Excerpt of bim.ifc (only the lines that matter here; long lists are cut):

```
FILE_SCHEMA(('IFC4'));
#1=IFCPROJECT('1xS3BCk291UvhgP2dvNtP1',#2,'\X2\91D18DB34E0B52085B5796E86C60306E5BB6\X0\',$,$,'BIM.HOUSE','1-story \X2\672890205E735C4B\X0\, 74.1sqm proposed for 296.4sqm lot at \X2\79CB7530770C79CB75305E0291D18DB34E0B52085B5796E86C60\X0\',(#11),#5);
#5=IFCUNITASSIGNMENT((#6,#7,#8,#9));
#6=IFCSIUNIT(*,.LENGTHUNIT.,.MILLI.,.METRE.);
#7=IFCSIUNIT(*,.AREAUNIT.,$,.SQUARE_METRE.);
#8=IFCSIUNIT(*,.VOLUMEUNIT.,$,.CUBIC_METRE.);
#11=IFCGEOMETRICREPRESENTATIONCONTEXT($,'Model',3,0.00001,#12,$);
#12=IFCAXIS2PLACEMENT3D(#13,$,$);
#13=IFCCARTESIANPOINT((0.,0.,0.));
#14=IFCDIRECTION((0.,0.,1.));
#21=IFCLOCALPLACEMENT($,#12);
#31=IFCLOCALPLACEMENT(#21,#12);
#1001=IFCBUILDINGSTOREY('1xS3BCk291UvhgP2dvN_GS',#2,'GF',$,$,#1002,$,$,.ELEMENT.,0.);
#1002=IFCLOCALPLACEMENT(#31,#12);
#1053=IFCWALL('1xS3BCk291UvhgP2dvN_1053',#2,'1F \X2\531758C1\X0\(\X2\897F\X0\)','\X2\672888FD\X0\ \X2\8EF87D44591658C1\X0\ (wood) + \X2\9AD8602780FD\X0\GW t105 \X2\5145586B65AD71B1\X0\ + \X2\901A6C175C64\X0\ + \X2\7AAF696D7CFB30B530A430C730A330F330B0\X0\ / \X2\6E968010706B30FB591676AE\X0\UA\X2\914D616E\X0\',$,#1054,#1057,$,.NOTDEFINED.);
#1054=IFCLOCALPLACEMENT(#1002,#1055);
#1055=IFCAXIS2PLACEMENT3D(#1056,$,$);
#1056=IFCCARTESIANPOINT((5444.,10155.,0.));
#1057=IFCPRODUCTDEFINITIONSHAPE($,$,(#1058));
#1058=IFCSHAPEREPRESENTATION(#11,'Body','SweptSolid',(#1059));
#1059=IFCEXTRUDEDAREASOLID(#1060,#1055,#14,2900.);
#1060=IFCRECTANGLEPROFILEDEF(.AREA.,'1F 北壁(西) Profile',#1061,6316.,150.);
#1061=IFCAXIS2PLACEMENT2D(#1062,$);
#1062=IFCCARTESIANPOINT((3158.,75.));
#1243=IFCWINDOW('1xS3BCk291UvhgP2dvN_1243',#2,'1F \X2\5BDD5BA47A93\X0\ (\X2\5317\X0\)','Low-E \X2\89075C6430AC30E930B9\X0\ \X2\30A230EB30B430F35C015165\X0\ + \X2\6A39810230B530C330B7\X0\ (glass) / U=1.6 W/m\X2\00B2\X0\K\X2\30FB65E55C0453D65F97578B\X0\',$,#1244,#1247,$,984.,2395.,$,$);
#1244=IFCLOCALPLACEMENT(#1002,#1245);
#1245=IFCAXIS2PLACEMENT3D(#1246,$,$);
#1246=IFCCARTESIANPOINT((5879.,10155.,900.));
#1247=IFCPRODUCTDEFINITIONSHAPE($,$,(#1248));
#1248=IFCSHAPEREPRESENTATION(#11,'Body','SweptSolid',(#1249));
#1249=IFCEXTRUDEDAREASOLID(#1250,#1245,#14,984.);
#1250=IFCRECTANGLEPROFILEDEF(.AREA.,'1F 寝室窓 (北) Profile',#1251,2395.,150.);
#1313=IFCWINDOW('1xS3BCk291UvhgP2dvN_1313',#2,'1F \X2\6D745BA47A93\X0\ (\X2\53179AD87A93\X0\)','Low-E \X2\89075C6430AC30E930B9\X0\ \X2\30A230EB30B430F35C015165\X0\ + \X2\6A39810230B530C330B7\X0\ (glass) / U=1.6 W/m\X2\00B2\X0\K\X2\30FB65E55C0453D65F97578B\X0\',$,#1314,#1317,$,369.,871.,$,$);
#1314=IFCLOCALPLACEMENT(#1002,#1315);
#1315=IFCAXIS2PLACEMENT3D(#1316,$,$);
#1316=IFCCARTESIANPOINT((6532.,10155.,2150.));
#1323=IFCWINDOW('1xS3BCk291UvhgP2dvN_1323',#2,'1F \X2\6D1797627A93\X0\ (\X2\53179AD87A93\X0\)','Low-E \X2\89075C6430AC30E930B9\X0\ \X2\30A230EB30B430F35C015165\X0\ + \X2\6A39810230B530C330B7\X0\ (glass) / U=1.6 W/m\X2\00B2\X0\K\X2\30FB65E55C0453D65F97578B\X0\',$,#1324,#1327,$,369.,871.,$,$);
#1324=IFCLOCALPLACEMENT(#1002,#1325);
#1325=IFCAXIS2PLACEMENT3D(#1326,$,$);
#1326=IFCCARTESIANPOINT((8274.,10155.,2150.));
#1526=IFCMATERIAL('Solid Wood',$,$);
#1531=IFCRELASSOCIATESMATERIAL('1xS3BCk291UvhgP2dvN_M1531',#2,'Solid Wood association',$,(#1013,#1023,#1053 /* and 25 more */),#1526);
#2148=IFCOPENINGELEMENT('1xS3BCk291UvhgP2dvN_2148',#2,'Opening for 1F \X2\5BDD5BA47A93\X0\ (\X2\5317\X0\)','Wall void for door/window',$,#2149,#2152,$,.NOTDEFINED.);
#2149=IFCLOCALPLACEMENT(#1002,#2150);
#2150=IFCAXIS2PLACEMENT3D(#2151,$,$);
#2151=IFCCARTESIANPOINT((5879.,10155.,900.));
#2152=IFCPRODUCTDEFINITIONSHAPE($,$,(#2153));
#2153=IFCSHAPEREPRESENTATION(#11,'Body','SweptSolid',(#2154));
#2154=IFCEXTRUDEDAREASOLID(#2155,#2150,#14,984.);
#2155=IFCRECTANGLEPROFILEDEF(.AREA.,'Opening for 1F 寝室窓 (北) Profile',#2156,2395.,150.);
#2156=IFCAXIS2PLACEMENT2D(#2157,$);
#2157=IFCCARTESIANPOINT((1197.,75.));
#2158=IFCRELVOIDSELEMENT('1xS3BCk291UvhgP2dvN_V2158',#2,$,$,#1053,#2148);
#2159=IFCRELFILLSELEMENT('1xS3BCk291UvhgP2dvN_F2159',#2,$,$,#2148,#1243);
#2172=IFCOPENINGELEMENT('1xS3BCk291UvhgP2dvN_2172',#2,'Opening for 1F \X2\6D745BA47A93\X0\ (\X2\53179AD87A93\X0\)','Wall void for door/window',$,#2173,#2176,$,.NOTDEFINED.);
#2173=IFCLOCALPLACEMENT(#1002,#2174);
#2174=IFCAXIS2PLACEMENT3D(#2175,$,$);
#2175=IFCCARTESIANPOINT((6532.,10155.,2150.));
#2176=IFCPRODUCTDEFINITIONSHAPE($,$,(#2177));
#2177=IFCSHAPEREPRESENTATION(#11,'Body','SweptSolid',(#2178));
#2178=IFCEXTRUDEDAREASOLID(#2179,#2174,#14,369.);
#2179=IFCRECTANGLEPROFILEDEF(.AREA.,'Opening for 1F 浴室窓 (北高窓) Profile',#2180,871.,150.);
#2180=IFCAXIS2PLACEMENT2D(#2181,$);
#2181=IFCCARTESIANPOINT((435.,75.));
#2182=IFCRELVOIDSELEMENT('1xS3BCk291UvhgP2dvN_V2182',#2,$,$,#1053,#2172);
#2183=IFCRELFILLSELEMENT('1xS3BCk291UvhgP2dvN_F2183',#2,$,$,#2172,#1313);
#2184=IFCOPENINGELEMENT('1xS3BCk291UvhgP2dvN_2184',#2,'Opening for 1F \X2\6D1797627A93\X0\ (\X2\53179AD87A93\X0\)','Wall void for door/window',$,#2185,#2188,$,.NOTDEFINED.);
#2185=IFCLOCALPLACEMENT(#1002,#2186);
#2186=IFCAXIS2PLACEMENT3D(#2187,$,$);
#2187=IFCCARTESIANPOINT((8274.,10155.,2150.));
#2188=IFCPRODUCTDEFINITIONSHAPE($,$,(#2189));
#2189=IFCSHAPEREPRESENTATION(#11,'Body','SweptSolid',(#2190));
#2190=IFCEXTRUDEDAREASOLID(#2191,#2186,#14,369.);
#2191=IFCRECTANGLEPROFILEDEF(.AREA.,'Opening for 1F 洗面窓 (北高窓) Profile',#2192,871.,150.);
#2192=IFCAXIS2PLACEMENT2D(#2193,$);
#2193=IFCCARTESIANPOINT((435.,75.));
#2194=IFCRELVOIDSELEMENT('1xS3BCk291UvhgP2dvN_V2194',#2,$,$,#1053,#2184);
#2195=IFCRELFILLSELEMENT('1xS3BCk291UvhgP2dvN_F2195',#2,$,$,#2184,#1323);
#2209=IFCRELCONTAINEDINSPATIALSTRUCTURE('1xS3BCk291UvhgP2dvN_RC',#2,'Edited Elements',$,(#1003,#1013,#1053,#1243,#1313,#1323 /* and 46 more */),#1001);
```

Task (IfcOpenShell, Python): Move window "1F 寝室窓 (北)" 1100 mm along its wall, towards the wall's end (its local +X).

```python
import ifcopenshell
import ifcopenshell.api.geometry
import ifcopenshell.util.placement

model = ifcopenshell.open("bim.ifc")

window = model.by_guid("1xS3BCk291UvhgP2dvN_1243")
opening = window.FillsVoids[0].RelatingOpeningElement
wall = opening.VoidsElements[0].RelatingBuildingElement

wall_matrix = ifcopenshell.util.placement.get_local_placement(wall.ObjectPlacement)
shift = wall_matrix[:3, 0] * 1100.0
before = ifcopenshell.util.placement.get_local_placement(window.ObjectPlacement)[:3, 3].copy()

# The window is not placed relative to its opening, so move both.
for product in (opening, window):
    matrix = ifcopenshell.util.placement.get_local_placement(product.ObjectPlacement)
    matrix[:3, 3] += shift
    ifcopenshell.api.geometry.edit_object_placement(model, product=product, matrix=matrix, is_si=False)

after = ifcopenshell.util.placement.get_local_placement(window.ObjectPlacement)[:3, 3]
print("window moved by", (after - before).round(3) + 0.0)

model.write("bim_edited.ifc")
```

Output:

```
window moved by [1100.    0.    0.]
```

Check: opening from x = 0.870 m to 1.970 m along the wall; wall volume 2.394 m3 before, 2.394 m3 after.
